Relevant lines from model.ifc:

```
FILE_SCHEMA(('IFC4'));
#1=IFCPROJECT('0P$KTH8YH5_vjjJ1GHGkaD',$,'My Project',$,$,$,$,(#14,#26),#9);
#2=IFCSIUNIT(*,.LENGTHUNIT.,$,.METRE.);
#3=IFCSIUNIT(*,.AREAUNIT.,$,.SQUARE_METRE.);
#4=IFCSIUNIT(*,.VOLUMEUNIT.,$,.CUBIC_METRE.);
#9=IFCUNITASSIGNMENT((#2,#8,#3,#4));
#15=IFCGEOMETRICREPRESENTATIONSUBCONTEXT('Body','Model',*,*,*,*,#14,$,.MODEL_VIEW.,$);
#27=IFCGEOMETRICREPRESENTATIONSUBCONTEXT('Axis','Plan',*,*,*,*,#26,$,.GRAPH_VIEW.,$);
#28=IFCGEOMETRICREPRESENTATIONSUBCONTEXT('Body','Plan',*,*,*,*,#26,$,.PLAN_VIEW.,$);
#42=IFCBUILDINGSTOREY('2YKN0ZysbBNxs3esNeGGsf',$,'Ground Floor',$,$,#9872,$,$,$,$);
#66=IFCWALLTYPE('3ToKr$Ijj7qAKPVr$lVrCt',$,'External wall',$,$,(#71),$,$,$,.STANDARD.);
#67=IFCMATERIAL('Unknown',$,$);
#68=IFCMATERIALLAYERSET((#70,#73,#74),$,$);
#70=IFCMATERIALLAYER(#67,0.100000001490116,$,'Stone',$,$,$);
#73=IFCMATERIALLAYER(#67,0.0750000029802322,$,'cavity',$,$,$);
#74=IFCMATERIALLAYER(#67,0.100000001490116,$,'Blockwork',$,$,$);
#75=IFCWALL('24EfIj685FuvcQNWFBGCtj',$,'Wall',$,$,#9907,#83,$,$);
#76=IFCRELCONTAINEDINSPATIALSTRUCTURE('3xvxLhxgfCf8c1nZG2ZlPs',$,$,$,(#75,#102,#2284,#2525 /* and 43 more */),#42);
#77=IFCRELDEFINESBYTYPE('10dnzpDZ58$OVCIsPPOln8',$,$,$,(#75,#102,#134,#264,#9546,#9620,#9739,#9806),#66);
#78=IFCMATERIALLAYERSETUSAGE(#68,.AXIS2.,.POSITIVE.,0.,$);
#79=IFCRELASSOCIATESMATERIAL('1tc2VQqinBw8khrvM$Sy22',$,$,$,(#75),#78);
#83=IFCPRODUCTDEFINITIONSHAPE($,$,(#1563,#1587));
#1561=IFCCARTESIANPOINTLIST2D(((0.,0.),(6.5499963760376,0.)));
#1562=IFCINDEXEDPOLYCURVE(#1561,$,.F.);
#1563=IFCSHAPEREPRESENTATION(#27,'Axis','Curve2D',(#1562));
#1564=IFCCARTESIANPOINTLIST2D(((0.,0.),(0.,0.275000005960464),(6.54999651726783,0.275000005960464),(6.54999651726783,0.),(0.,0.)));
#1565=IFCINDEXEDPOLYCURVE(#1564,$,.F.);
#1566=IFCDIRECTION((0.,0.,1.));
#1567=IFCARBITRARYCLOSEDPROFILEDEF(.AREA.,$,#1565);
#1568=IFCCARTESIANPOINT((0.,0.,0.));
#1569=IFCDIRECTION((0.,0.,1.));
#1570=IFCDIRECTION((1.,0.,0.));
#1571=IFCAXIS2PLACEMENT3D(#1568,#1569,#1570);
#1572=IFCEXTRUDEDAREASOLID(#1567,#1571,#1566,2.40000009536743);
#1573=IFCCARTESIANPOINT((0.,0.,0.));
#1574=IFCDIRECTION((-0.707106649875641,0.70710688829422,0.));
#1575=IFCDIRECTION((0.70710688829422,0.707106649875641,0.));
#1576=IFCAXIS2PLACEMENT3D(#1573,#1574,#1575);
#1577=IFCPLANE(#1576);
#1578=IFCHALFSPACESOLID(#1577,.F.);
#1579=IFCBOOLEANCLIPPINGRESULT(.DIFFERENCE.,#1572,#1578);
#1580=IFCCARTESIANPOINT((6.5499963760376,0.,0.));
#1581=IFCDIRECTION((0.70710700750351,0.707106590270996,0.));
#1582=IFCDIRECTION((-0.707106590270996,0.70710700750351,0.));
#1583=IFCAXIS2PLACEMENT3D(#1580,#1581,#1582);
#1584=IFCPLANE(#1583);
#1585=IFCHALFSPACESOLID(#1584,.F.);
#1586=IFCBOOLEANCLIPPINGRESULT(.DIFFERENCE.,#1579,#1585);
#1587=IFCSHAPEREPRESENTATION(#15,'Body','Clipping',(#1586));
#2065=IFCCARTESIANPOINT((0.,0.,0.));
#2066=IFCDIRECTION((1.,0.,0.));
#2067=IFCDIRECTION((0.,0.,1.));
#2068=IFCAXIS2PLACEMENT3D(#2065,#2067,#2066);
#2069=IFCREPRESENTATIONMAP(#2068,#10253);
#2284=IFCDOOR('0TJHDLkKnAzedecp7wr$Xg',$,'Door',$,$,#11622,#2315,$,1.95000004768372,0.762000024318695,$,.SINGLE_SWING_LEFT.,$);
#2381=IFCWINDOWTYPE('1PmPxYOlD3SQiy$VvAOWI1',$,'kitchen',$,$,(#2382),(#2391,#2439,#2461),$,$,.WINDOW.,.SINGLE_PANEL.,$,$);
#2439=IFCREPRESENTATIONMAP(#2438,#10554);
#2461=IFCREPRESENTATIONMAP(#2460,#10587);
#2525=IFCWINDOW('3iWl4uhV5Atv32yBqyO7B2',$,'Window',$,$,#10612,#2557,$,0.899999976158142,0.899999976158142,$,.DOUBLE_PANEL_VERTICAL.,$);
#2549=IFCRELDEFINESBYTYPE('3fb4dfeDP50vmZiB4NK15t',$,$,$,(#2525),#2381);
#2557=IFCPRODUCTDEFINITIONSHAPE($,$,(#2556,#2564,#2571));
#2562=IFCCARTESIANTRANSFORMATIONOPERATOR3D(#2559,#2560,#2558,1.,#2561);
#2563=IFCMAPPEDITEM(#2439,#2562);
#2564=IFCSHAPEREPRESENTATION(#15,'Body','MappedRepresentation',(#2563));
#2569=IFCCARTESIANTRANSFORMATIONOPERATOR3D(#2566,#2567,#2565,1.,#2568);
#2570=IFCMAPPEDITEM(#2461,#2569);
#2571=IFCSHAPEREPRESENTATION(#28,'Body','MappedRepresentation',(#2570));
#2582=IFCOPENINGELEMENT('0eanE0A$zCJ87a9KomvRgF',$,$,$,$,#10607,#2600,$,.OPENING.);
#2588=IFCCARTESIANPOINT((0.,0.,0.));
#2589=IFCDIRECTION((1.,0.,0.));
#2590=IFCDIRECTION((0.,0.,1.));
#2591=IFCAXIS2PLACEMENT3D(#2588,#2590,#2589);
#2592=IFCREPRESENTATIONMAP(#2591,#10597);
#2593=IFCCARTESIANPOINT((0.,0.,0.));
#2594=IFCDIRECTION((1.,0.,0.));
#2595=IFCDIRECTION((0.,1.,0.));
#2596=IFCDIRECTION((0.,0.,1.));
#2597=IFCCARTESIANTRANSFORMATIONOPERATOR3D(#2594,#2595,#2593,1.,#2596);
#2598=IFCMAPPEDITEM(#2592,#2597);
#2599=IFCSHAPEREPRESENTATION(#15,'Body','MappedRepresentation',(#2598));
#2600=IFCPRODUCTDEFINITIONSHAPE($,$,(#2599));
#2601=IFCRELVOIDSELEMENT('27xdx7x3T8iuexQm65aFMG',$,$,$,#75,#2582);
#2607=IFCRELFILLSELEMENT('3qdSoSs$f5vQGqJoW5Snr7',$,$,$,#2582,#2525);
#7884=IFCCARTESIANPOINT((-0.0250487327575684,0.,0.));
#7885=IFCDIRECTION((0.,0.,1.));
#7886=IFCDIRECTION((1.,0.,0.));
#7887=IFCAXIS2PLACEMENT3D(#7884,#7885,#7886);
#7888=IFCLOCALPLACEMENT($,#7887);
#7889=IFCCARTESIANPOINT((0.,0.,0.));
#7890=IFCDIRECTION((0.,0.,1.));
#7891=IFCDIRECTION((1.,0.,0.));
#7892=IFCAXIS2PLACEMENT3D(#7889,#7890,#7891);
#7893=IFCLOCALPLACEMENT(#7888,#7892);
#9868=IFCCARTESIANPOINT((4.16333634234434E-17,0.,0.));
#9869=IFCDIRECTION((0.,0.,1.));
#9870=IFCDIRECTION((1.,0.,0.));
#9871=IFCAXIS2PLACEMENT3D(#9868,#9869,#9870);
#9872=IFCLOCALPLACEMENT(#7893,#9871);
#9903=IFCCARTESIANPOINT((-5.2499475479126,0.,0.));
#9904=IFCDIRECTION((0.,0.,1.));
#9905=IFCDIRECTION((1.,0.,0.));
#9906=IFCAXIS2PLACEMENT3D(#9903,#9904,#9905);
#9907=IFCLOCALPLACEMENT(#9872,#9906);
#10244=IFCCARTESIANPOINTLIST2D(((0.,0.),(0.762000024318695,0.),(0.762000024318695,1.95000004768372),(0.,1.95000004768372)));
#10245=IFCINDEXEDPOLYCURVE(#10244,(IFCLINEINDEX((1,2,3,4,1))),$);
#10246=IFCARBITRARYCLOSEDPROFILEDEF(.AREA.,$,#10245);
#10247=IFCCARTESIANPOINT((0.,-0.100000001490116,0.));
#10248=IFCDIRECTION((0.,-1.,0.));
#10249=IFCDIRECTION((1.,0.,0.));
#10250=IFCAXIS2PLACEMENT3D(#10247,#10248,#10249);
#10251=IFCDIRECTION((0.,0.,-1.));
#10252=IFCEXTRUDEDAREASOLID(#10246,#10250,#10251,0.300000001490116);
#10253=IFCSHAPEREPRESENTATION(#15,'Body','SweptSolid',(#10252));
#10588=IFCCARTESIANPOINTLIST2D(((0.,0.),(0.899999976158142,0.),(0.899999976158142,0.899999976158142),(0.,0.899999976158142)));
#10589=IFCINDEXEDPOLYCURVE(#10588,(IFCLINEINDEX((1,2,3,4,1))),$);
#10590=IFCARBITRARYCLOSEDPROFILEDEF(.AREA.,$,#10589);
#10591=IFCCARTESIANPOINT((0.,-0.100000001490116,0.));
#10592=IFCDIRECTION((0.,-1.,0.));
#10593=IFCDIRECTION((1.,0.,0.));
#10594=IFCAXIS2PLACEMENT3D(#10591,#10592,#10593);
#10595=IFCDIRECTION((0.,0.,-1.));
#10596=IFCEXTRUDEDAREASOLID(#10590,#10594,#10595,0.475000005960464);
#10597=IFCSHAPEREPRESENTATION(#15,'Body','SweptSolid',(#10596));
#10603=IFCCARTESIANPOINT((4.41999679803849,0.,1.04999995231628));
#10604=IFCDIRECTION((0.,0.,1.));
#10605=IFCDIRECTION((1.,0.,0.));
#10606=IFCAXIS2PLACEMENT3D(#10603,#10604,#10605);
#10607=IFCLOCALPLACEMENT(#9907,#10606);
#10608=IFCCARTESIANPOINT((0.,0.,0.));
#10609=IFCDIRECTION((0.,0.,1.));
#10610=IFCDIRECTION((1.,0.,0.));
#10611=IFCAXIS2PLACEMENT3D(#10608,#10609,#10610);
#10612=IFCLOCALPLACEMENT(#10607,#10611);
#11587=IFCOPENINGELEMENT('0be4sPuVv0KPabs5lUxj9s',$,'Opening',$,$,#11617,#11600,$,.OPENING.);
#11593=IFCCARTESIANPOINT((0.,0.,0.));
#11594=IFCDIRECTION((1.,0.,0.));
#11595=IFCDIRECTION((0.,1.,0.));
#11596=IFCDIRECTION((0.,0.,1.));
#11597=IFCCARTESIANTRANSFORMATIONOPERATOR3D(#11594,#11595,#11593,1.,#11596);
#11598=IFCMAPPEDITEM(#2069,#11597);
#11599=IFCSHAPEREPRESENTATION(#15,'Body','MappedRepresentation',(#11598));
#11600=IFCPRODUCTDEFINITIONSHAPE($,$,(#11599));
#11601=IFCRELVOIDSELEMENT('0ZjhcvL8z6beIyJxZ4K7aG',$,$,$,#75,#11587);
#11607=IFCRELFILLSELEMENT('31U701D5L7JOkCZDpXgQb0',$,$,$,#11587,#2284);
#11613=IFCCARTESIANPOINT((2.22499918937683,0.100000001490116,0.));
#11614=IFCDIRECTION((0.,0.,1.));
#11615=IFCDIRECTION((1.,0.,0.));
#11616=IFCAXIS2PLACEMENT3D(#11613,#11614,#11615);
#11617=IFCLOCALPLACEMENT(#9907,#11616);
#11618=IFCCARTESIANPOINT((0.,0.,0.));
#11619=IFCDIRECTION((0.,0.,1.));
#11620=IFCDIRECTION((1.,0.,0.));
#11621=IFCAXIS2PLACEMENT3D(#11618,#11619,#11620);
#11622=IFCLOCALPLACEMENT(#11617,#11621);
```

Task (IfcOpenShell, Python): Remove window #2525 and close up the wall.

```python
import ifcopenshell
import ifcopenshell.api.feature
import ifcopenshell.api.root
import ifcopenshell.geom
import ifcopenshell.util.shape

model = ifcopenshell.open("model.ifc")
settings = ifcopenshell.geom.settings()


def volume(element):
    """Net volume in cubic metres, openings subtracted."""
    shape = ifcopenshell.geom.create_shape(settings, element)
    return ifcopenshell.util.shape.get_volume(shape.geometry)


window = model.by_guid("3iWl4uhV5Atv32yBqyO7B2")
opening = window.FillsVoids[0].RelatingOpeningElement
wall = opening.VoidsElements[0].RelatingBuildingElement
before = volume(wall)

ifcopenshell.api.root.remove_product(model, product=window)
ifcopenshell.api.feature.remove_feature(model, feature=opening)

after = volume(wall)

print(f"wall volume {before:.3f} -> {after:.3f} m3")

model.write("model_rev.ifc")
```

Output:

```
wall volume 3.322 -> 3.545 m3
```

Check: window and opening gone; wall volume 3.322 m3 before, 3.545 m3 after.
